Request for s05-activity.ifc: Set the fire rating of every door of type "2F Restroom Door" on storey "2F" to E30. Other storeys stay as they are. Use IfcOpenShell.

First a look at what the model holds.

```python
import ifcopenshell
import ifcopenshell.util.element

model = ifcopenshell.open("s05-activity.ifc")
print(model.schema)
storey = next(s for s in model.by_type("IfcBuildingStorey") if s.Name == "2F")
doors = [e for e in ifcopenshell.util.element.get_decomposition(storey) if e.is_a("IfcDoor")]
seen = {}
for e in doors:
    element_type = ifcopenshell.util.element.get_type(e)
    key = (element_type.Name if element_type != e and element_type else None, ifcopenshell.util.element.get_pset(e, "Pset_DoorCommon", "FireRating"))
    seen[key] = seen.get(key, 0) + 1
for (name, value), count in sorted(seen.items(), key=str):
    print(count, "x", name, "|", value)
```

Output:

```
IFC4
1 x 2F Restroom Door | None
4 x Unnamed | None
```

```python
import ifcopenshell
import ifcopenshell.api.pset
import ifcopenshell.util.element

model = ifcopenshell.open("s05-activity.ifc")

storey = next(s for s in model.by_type("IfcBuildingStorey") if s.Name == "2F")
doors = [e for e in ifcopenshell.util.element.get_decomposition(storey) if e.is_a("IfcDoor")]

count = 0
for e in doors:
    element_type = ifcopenshell.util.element.get_type(e)
    if element_type in (None, e) or element_type.Name != "2F Restroom Door":
        continue
    # add_pset returns the element's existing set when there is one.
    pset = ifcopenshell.api.pset.add_pset(model, product=e, name="Pset_DoorCommon")
    ifcopenshell.api.pset.edit_pset(model, pset=pset, properties={"FireRating": "E30"})
    count += 1

print(count, "doors updated")

model.write("s05-activity_v2.ifc")
```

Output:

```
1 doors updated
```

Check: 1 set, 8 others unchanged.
